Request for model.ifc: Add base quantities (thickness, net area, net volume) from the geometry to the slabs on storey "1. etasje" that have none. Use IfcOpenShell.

First a look at what the model holds.

```python
import ifcopenshell
import ifcopenshell.util.element
import ifcopenshell.util.unit

model = ifcopenshell.open("model.ifc")
print(model.schema)
for unit_type in ("LENGTHUNIT", "AREAUNIT", "VOLUMEUNIT"):
    print(unit_type, ifcopenshell.util.unit.calculate_unit_scale(model, unit_type))
storey = next(s for s in model.by_type("IfcBuildingStorey") if s.Name == "1. etasje")
slabs = [e for e in ifcopenshell.util.element.get_decomposition(storey) if e.is_a("IfcSlab")]
for e in sorted(slabs, key=lambda e: e.id()):
    print(e.id(), e.is_a(), e.Name, list(ifcopenshell.util.element.get_psets(e, qtos_only=True)), sep=" | ")
```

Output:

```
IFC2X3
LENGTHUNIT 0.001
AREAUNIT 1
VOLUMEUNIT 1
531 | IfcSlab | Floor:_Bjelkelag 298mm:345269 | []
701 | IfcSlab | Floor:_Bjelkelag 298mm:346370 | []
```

```python
import ifcopenshell
import ifcopenshell.api.pset
import ifcopenshell.geom
import ifcopenshell.util.element
import ifcopenshell.util.shape
import ifcopenshell.util.unit

model = ifcopenshell.open("model.ifc")
unit_scale = ifcopenshell.util.unit.calculate_unit_scale(model)
area_scale = ifcopenshell.util.unit.calculate_unit_scale(model, "AREAUNIT")
volume_scale = ifcopenshell.util.unit.calculate_unit_scale(model, "VOLUMEUNIT")
settings = ifcopenshell.geom.settings()

storey = next(s for s in model.by_type("IfcBuildingStorey") if s.Name == "1. etasje")
slabs = [e for e in ifcopenshell.util.element.get_decomposition(storey) if e.is_a("IfcSlab")]

for e in sorted(slabs, key=lambda e: e.id()):
    if ifcopenshell.util.element.get_psets(e, qtos_only=True, should_inherit=False):
        continue
    # Geometry comes back in metres, in the element's own axes.
    shape = ifcopenshell.geom.create_shape(settings, e)
    values = {
        "Width": ifcopenshell.util.shape.get_z(shape.geometry) / unit_scale,
        "NetArea": ifcopenshell.util.shape.get_footprint_area(shape.geometry) / area_scale,
        "NetVolume": ifcopenshell.util.shape.get_volume(shape.geometry) / volume_scale,
    }
    qto = ifcopenshell.api.pset.add_qto(model, product=e, name="BaseQuantities")
    ifcopenshell.api.pset.edit_qto(model, qto=qto, properties=values)
    print(e.id(), {k: round(v, 3) for k, v in values.items()})

model.write("model_v2.ifc")
```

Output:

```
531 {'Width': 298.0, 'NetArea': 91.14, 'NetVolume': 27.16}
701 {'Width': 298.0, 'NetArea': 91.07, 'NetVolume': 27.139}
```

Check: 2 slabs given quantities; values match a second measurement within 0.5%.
